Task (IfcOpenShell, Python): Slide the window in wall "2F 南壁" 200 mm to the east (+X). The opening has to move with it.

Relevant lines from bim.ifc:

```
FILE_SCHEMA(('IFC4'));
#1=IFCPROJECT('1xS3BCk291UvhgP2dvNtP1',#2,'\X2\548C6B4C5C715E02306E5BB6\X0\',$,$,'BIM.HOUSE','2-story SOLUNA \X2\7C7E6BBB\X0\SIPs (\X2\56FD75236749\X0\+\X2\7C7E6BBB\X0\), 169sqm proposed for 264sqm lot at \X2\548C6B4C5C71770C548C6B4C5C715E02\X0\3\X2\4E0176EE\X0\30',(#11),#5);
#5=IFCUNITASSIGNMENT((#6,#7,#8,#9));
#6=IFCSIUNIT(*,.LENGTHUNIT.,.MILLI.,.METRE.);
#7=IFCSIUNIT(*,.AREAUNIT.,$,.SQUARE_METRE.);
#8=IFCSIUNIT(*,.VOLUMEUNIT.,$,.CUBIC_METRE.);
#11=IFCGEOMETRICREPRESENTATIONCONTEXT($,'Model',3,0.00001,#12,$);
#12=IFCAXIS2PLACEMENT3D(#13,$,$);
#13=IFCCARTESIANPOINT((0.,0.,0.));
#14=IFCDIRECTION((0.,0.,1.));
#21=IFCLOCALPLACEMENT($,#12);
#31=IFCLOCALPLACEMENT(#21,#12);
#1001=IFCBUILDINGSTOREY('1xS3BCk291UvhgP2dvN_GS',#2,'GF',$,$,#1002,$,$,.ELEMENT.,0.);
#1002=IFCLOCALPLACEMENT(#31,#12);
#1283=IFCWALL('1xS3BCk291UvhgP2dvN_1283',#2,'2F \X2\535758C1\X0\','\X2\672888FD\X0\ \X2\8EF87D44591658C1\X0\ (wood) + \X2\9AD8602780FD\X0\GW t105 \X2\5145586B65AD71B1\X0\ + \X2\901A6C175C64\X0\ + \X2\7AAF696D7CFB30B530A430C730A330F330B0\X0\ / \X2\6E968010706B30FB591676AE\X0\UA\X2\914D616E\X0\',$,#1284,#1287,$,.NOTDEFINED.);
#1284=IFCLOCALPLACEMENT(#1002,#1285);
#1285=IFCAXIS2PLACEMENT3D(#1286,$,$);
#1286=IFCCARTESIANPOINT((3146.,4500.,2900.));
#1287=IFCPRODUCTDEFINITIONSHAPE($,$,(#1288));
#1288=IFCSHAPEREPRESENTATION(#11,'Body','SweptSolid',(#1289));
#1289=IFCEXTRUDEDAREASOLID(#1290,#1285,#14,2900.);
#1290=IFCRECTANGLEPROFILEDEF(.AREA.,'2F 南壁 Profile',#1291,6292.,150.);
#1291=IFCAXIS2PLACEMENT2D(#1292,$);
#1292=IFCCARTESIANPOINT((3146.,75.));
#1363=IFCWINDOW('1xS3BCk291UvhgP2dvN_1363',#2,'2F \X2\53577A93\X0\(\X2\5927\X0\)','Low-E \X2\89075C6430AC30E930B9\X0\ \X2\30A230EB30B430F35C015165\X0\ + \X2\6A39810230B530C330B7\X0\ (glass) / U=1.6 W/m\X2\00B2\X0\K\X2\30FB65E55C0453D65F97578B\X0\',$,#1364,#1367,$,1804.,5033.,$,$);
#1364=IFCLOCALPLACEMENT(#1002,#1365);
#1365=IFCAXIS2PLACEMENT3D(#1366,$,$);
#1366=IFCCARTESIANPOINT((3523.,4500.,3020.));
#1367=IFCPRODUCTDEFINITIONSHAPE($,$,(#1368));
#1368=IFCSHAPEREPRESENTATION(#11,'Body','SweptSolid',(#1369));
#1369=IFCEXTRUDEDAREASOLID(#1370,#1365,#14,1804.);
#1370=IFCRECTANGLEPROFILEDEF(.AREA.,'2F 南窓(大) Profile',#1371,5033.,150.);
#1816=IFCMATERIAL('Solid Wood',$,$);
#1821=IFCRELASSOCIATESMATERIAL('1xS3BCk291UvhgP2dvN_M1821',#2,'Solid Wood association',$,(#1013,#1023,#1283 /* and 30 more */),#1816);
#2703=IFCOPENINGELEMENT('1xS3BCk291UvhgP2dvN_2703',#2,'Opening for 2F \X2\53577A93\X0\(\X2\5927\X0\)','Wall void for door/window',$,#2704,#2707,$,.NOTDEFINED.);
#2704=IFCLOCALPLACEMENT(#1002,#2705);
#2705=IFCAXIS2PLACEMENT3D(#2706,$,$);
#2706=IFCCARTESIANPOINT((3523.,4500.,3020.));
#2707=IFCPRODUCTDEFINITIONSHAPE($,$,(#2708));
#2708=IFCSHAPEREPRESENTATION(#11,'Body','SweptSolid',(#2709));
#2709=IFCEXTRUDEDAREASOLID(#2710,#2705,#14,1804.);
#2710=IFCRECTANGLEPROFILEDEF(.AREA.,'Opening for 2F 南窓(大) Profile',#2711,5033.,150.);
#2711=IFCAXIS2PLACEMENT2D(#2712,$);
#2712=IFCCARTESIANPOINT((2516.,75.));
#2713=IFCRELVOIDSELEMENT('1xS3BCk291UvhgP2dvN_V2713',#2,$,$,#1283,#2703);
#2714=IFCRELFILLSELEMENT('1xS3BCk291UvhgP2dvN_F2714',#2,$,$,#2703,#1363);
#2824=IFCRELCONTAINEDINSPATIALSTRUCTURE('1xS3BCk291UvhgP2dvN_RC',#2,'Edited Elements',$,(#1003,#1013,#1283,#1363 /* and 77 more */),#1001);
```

```python
import ifcopenshell
import ifcopenshell.api.geometry
import ifcopenshell.util.placement

model = ifcopenshell.open("bim.ifc")

window = model.by_guid("1xS3BCk291UvhgP2dvN_1363")
opening = window.FillsVoids[0].RelatingOpeningElement
wall = opening.VoidsElements[0].RelatingBuildingElement

wall_matrix = ifcopenshell.util.placement.get_local_placement(wall.ObjectPlacement)
shift = wall_matrix[:3, 0] * 200.0
before = ifcopenshell.util.placement.get_local_placement(window.ObjectPlacement)[:3, 3].copy()

# The window is not placed relative to its opening, so move both.
for product in (opening, window):
    matrix = ifcopenshell.util.placement.get_local_placement(product.ObjectPlacement)
    matrix[:3, 3] += shift
    ifcopenshell.api.geometry.edit_object_placement(model, product=product, matrix=matrix, is_si=False)

after = ifcopenshell.util.placement.get_local_placement(window.ObjectPlacement)[:3, 3]
print("window moved by", (after - before).round(3) + 0.0)

model.write("bim_edited.ifc")
```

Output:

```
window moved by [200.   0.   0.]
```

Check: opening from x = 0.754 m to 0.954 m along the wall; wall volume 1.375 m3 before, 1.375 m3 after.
